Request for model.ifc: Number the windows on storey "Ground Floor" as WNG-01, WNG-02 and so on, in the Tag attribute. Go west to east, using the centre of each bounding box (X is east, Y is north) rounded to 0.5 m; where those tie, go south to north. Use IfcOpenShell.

First a look at what the model holds.

```python
import ifcopenshell
import ifcopenshell.util.element
import ifcopenshell.util.placement

model = ifcopenshell.open("model.ifc")
print(model.schema)
storey = next(s for s in model.by_type("IfcBuildingStorey") if s.Name == "Ground Floor")
windows = [e for e in ifcopenshell.util.element.get_decomposition(storey) if e.is_a("IfcWindow")]
for e in sorted(windows, key=lambda e: e.id()):
    origin = ifcopenshell.util.placement.get_local_placement(e.ObjectPlacement)[:3, 3]
    print(e.id(), e.Tag, e.Name, origin.round(2) + 0.0, sep=" | ")
```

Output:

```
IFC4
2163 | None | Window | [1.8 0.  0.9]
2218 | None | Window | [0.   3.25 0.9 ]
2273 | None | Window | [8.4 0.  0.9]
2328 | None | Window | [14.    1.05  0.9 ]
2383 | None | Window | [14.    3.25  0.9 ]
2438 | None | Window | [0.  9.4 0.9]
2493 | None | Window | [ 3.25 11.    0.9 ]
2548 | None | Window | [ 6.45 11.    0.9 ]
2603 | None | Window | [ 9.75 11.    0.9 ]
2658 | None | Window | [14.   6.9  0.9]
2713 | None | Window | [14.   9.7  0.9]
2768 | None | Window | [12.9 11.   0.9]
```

```python
import ifcopenshell
import ifcopenshell.geom
import ifcopenshell.util.element
import ifcopenshell.util.shape

model = ifcopenshell.open("model.ifc")
settings = ifcopenshell.geom.settings()
settings.set("use-world-coords", True)


def centre(element):
    shape = ifcopenshell.geom.create_shape(settings, element)
    return ifcopenshell.util.shape.get_bbox_centroid(shape.geometry)


storey = next(s for s in model.by_type("IfcBuildingStorey") if s.Name == "Ground Floor")
windows = [e for e in ifcopenshell.util.element.get_decomposition(storey) if e.is_a("IfcWindow")]

# Insertion points can sit at a corner or the storey origin, so sort by the geometry (in metres).
centres = {e: centre(e) for e in windows}
windows.sort(key=lambda e: (round(centres[e][0] / 0.5), centres[e][1]))

for i, e in enumerate(windows, start=1):
    number = f"WNG-{i:02d}"
    e.Tag = number
    print(e.id(), number)

model.write("model_edited.ifc")
```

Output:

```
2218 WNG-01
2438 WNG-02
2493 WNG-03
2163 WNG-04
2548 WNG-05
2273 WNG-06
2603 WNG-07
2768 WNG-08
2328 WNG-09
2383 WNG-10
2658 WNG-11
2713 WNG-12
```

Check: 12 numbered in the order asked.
